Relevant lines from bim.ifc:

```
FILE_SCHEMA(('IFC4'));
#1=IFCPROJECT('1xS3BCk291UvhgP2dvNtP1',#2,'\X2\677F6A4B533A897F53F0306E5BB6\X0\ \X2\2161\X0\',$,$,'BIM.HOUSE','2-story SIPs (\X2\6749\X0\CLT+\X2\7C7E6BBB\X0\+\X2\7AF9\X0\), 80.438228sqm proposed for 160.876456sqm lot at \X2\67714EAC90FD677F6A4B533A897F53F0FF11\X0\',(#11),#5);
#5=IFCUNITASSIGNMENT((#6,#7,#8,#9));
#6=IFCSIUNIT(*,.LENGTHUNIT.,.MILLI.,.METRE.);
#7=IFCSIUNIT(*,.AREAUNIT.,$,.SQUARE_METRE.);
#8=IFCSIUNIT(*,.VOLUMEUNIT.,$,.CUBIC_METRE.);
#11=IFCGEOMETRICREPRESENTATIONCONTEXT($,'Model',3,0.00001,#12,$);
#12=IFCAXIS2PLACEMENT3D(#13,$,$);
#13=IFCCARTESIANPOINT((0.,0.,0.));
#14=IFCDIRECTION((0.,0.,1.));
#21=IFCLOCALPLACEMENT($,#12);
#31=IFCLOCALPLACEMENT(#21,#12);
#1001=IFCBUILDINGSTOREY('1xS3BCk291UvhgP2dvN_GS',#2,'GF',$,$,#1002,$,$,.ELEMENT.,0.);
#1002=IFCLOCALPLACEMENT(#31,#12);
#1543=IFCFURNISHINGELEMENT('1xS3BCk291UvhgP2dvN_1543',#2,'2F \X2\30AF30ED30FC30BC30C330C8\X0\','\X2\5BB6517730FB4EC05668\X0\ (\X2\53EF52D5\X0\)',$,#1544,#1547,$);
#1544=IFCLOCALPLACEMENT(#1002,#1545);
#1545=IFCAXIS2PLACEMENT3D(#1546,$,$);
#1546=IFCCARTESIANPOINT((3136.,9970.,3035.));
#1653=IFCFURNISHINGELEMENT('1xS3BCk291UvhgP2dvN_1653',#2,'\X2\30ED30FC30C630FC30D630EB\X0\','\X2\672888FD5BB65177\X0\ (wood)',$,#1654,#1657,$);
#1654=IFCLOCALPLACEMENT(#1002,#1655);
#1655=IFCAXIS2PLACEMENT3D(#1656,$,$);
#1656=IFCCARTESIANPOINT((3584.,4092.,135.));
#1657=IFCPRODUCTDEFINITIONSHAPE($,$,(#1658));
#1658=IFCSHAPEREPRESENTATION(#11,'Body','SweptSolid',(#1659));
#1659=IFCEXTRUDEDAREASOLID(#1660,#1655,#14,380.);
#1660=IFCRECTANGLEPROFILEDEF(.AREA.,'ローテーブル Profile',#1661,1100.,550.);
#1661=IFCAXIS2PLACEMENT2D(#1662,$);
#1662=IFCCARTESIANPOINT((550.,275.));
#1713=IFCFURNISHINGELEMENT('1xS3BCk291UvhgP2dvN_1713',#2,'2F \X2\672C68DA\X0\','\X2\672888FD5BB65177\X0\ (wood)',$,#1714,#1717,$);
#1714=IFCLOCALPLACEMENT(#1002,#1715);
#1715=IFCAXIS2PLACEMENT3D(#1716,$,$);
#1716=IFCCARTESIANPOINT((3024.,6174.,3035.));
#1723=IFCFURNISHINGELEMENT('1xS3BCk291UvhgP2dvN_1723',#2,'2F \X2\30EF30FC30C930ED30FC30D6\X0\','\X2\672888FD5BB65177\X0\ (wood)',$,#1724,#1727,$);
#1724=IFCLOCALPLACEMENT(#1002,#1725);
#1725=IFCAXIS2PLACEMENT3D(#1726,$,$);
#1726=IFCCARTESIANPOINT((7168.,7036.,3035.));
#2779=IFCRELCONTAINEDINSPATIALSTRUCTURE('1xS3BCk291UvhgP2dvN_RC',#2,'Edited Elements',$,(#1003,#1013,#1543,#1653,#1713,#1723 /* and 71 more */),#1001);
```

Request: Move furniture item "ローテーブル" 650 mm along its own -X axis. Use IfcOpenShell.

```python
import ifcopenshell
import ifcopenshell.api.geometry
import ifcopenshell.util.placement

model = ifcopenshell.open("bim.ifc")

item = model.by_guid("1xS3BCk291UvhgP2dvN_1653")
matrix = ifcopenshell.util.placement.get_local_placement(item.ObjectPlacement)
matrix[:3, 3] -= matrix[:3, 0] * 650.0
ifcopenshell.api.geometry.edit_object_placement(model, product=item, matrix=matrix, is_si=False)

print(ifcopenshell.util.placement.get_local_placement(item.ObjectPlacement).round(3) + 0.0)

model.write("bim-out.ifc")
```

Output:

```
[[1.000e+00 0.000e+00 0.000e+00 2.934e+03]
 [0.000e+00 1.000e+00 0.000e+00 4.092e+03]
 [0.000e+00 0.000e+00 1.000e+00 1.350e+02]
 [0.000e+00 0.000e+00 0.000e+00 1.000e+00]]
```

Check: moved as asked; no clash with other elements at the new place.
